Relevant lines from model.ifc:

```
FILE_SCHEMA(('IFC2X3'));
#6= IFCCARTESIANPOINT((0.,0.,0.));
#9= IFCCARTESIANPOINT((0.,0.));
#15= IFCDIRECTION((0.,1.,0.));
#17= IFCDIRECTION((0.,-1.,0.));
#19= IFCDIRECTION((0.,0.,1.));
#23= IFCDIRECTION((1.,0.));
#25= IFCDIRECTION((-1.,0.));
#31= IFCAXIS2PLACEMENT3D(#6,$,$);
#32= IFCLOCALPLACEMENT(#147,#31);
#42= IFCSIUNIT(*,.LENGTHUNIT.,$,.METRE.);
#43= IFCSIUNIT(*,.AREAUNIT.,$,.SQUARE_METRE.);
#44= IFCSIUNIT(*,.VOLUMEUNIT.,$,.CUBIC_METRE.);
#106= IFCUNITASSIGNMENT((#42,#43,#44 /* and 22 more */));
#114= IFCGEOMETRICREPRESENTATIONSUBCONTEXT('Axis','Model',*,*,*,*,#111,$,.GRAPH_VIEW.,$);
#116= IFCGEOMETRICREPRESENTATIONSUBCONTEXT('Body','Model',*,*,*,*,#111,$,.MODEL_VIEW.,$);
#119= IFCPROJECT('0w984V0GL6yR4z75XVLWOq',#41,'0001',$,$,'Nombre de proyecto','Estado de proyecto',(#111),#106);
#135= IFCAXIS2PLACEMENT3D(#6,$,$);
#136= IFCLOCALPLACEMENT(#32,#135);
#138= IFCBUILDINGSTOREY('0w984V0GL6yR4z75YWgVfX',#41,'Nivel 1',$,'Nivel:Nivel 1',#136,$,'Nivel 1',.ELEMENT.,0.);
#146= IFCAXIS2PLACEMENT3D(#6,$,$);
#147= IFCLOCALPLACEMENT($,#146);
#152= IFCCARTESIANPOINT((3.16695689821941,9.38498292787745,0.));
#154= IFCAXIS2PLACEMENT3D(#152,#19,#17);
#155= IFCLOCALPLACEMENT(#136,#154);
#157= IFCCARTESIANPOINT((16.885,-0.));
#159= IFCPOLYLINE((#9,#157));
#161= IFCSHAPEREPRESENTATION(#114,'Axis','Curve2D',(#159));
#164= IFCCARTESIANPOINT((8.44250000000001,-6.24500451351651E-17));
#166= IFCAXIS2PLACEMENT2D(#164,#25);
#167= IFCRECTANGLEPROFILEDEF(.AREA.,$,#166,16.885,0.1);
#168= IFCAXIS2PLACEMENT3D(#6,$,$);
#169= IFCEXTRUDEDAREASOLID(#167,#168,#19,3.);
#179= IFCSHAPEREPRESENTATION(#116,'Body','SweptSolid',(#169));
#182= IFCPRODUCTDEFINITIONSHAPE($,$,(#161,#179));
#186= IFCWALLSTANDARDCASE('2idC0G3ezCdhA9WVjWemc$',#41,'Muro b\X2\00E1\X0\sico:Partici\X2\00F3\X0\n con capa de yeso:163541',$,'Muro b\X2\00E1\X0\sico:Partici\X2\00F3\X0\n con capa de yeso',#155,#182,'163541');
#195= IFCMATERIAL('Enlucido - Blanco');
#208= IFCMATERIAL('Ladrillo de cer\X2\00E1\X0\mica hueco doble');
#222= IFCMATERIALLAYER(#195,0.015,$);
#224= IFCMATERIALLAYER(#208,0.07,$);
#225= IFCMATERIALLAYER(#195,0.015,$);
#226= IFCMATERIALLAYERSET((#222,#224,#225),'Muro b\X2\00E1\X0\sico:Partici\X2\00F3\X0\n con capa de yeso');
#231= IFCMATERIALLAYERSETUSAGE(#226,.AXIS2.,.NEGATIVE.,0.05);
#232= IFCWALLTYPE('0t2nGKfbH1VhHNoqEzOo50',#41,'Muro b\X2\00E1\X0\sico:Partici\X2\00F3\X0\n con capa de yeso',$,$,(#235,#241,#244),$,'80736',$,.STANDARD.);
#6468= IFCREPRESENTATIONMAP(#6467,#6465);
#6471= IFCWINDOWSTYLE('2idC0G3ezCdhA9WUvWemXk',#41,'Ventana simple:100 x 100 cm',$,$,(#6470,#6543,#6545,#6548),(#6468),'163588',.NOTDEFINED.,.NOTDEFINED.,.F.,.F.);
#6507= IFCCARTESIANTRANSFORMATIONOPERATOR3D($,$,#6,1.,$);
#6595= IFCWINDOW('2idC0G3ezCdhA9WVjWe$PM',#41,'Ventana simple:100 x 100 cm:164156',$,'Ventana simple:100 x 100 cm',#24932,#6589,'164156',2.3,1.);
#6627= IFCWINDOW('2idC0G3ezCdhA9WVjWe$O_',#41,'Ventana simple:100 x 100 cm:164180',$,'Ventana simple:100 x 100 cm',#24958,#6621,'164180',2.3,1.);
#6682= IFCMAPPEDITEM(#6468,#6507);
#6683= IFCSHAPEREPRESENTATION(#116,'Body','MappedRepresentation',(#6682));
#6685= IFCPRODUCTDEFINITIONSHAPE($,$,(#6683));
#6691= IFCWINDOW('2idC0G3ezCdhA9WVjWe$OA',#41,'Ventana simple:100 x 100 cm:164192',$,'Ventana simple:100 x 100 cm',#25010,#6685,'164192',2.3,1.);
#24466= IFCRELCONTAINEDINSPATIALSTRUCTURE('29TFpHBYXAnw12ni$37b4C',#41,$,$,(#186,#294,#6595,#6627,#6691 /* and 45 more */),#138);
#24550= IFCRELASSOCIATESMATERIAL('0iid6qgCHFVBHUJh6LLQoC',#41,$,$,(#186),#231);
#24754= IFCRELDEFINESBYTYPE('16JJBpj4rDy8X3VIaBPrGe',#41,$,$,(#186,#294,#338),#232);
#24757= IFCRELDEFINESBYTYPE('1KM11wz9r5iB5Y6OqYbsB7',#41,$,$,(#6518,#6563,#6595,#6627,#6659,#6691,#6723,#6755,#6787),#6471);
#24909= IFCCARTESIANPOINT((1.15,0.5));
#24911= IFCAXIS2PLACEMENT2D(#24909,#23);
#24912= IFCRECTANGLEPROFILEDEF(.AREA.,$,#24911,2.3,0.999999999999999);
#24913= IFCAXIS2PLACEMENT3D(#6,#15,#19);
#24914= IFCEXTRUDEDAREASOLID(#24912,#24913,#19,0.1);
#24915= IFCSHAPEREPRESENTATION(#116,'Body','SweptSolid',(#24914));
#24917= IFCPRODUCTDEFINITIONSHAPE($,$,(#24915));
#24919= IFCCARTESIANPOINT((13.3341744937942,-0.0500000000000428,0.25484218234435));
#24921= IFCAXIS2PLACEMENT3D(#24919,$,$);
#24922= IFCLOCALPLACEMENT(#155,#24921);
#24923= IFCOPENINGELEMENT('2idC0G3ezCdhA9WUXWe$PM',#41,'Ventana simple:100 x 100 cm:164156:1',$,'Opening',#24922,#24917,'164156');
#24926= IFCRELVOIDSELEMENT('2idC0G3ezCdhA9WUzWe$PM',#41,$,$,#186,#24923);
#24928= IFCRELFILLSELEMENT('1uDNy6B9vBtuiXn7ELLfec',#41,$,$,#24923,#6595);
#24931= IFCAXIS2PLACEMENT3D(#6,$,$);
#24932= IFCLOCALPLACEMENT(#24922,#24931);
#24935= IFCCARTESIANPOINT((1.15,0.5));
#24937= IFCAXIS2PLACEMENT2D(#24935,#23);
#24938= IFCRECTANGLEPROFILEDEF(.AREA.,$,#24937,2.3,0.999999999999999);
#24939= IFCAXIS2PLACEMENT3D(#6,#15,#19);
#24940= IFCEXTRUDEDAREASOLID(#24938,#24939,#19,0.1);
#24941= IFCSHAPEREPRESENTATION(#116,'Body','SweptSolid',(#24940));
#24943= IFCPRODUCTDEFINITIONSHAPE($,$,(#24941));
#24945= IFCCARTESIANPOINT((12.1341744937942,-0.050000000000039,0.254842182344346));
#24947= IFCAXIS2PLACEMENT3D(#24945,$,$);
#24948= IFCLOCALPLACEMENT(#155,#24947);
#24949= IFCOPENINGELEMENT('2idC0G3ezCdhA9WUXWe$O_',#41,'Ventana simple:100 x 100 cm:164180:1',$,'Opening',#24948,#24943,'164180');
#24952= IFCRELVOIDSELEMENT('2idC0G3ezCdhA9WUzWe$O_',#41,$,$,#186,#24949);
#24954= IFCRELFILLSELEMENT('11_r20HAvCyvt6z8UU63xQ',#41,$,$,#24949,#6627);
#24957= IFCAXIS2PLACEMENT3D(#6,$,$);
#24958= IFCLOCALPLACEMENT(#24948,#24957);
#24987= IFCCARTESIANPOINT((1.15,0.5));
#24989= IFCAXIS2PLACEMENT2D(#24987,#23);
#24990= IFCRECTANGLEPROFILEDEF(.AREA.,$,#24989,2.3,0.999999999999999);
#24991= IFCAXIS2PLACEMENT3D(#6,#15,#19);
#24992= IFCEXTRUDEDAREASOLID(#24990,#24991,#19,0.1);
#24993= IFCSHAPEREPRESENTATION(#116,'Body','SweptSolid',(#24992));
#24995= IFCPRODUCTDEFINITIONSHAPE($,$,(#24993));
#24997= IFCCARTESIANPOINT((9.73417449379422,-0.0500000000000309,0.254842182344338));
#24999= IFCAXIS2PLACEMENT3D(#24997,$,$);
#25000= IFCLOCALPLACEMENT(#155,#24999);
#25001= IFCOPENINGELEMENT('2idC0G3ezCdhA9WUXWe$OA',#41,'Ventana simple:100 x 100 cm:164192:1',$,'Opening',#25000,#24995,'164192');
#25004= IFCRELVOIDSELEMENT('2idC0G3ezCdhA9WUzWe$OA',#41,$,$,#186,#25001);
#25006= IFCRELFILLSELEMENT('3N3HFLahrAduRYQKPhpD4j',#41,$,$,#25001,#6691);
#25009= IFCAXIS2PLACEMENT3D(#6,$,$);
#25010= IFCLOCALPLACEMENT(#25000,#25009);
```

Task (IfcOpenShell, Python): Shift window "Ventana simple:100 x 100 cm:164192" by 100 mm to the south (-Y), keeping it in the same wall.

```python
import ifcopenshell
import ifcopenshell.api.geometry
import ifcopenshell.util.placement

model = ifcopenshell.open("model.ifc")

window = model.by_id(6691)
opening = window.FillsVoids[0].RelatingOpeningElement
wall = opening.VoidsElements[0].RelatingBuildingElement

wall_matrix = ifcopenshell.util.placement.get_local_placement(wall.ObjectPlacement)
shift = wall_matrix[:3, 0] * 0.1
before = ifcopenshell.util.placement.get_local_placement(window.ObjectPlacement)[:3, 3].copy()

# The window is placed relative to its opening, so it follows when the opening moves.
matrix = ifcopenshell.util.placement.get_local_placement(opening.ObjectPlacement)
matrix[:3, 3] += shift
ifcopenshell.api.geometry.edit_object_placement(
    model, product=opening, matrix=matrix, is_si=False, should_transform_children=True
)

after = ifcopenshell.util.placement.get_local_placement(window.ObjectPlacement)[:3, 3]
print("window moved by", (after - before).round(3) + 0.0)

model.write("model_updated.ifc")
```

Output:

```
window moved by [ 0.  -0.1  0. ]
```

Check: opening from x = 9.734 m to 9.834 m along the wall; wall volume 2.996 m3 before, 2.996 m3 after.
